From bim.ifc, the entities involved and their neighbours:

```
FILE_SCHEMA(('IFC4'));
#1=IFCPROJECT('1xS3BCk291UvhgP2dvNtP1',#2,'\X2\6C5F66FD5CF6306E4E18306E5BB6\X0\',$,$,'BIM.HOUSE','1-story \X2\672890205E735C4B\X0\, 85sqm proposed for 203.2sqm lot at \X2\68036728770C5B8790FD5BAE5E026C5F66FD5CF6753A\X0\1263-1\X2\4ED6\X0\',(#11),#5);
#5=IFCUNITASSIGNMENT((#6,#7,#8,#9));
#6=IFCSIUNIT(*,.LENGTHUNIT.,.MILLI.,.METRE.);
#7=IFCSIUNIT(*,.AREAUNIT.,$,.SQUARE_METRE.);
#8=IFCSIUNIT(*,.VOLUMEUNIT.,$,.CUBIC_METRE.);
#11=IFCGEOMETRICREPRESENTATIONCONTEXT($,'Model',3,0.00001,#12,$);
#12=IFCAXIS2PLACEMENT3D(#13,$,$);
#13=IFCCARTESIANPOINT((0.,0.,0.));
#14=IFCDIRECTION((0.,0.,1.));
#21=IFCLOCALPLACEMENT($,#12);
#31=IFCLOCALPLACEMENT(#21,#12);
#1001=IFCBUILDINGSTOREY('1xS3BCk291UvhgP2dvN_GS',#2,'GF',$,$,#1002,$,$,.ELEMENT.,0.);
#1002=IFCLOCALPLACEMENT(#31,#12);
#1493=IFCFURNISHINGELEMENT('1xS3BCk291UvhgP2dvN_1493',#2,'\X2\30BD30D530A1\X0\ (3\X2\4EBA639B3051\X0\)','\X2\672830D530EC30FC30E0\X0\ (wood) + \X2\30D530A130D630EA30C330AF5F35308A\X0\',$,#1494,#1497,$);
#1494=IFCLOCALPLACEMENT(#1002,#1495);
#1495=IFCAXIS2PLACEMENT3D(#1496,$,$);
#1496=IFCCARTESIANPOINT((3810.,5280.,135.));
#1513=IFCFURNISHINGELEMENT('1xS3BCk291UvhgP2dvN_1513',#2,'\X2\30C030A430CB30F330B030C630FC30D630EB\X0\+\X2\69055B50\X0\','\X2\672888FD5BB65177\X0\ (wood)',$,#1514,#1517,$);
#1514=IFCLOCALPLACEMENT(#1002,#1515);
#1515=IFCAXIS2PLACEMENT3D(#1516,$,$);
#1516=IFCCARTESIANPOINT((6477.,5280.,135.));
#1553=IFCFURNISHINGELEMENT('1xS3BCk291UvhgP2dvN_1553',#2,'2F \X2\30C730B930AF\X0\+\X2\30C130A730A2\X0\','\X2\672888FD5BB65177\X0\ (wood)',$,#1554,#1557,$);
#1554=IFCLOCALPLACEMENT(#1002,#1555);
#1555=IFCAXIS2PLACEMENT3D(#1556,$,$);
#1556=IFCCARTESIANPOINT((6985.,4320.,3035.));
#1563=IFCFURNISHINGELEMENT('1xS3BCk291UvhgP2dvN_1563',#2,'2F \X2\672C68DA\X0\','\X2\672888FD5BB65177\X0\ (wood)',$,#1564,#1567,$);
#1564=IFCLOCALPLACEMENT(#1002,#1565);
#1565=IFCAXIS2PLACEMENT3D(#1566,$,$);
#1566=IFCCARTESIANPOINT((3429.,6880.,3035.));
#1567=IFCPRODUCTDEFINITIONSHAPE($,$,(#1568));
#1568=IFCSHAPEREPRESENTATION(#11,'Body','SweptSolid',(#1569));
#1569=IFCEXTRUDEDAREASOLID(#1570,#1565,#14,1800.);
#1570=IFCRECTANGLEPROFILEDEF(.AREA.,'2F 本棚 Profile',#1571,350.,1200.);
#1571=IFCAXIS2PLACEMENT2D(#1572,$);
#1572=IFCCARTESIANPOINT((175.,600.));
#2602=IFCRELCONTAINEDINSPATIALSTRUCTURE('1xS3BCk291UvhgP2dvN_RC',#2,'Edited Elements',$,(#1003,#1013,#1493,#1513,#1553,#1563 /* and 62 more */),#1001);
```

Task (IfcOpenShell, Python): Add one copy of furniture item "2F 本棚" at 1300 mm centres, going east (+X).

```python
import numpy as np
import ifcopenshell
import ifcopenshell.api.geometry
import ifcopenshell.api.root
import ifcopenshell.util.element
import ifcopenshell.util.placement
import ifcopenshell.util.unit

model = ifcopenshell.open("bim.ifc")
unit_scale = ifcopenshell.util.unit.calculate_unit_scale(model)


def reuse_history(source, copy):
    """copy_class also copies each property set's owner history, people and application; keep the originals."""
    for rel in copy.IsDefinedBy:
        if rel.is_a("IfcRelDefinesByProperties") and (history := rel.RelatingPropertyDefinition.OwnerHistory):
            rel.RelatingPropertyDefinition.OwnerHistory = source.OwnerHistory
            ifcopenshell.util.element.remove_deep2(model, history)


source = model.by_guid("1xS3BCk291UvhgP2dvN_1563")
base = ifcopenshell.util.placement.get_local_placement(source.ObjectPlacement)
step = np.array([1.0, 0.0, 0.0]) * 1.3 / unit_scale

for i in range(1, 2):
    copy = ifcopenshell.api.root.copy_class(model, product=source)
    copy.Representation = ifcopenshell.util.element.copy_deep(
        model, source.Representation, exclude=["IfcGeometricRepresentationContext", "IfcRepresentationMap"]
    )
    reuse_history(source, copy)
    matrix = base.copy()
    matrix[:3, 3] += i * step
    print("added at", matrix[:3, 3].round(3) + 0.0)
    ifcopenshell.api.geometry.edit_object_placement(model, product=copy, matrix=matrix, is_si=False)

model.write("bim-out.ifc")
```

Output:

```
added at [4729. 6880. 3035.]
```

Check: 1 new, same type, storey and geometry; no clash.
